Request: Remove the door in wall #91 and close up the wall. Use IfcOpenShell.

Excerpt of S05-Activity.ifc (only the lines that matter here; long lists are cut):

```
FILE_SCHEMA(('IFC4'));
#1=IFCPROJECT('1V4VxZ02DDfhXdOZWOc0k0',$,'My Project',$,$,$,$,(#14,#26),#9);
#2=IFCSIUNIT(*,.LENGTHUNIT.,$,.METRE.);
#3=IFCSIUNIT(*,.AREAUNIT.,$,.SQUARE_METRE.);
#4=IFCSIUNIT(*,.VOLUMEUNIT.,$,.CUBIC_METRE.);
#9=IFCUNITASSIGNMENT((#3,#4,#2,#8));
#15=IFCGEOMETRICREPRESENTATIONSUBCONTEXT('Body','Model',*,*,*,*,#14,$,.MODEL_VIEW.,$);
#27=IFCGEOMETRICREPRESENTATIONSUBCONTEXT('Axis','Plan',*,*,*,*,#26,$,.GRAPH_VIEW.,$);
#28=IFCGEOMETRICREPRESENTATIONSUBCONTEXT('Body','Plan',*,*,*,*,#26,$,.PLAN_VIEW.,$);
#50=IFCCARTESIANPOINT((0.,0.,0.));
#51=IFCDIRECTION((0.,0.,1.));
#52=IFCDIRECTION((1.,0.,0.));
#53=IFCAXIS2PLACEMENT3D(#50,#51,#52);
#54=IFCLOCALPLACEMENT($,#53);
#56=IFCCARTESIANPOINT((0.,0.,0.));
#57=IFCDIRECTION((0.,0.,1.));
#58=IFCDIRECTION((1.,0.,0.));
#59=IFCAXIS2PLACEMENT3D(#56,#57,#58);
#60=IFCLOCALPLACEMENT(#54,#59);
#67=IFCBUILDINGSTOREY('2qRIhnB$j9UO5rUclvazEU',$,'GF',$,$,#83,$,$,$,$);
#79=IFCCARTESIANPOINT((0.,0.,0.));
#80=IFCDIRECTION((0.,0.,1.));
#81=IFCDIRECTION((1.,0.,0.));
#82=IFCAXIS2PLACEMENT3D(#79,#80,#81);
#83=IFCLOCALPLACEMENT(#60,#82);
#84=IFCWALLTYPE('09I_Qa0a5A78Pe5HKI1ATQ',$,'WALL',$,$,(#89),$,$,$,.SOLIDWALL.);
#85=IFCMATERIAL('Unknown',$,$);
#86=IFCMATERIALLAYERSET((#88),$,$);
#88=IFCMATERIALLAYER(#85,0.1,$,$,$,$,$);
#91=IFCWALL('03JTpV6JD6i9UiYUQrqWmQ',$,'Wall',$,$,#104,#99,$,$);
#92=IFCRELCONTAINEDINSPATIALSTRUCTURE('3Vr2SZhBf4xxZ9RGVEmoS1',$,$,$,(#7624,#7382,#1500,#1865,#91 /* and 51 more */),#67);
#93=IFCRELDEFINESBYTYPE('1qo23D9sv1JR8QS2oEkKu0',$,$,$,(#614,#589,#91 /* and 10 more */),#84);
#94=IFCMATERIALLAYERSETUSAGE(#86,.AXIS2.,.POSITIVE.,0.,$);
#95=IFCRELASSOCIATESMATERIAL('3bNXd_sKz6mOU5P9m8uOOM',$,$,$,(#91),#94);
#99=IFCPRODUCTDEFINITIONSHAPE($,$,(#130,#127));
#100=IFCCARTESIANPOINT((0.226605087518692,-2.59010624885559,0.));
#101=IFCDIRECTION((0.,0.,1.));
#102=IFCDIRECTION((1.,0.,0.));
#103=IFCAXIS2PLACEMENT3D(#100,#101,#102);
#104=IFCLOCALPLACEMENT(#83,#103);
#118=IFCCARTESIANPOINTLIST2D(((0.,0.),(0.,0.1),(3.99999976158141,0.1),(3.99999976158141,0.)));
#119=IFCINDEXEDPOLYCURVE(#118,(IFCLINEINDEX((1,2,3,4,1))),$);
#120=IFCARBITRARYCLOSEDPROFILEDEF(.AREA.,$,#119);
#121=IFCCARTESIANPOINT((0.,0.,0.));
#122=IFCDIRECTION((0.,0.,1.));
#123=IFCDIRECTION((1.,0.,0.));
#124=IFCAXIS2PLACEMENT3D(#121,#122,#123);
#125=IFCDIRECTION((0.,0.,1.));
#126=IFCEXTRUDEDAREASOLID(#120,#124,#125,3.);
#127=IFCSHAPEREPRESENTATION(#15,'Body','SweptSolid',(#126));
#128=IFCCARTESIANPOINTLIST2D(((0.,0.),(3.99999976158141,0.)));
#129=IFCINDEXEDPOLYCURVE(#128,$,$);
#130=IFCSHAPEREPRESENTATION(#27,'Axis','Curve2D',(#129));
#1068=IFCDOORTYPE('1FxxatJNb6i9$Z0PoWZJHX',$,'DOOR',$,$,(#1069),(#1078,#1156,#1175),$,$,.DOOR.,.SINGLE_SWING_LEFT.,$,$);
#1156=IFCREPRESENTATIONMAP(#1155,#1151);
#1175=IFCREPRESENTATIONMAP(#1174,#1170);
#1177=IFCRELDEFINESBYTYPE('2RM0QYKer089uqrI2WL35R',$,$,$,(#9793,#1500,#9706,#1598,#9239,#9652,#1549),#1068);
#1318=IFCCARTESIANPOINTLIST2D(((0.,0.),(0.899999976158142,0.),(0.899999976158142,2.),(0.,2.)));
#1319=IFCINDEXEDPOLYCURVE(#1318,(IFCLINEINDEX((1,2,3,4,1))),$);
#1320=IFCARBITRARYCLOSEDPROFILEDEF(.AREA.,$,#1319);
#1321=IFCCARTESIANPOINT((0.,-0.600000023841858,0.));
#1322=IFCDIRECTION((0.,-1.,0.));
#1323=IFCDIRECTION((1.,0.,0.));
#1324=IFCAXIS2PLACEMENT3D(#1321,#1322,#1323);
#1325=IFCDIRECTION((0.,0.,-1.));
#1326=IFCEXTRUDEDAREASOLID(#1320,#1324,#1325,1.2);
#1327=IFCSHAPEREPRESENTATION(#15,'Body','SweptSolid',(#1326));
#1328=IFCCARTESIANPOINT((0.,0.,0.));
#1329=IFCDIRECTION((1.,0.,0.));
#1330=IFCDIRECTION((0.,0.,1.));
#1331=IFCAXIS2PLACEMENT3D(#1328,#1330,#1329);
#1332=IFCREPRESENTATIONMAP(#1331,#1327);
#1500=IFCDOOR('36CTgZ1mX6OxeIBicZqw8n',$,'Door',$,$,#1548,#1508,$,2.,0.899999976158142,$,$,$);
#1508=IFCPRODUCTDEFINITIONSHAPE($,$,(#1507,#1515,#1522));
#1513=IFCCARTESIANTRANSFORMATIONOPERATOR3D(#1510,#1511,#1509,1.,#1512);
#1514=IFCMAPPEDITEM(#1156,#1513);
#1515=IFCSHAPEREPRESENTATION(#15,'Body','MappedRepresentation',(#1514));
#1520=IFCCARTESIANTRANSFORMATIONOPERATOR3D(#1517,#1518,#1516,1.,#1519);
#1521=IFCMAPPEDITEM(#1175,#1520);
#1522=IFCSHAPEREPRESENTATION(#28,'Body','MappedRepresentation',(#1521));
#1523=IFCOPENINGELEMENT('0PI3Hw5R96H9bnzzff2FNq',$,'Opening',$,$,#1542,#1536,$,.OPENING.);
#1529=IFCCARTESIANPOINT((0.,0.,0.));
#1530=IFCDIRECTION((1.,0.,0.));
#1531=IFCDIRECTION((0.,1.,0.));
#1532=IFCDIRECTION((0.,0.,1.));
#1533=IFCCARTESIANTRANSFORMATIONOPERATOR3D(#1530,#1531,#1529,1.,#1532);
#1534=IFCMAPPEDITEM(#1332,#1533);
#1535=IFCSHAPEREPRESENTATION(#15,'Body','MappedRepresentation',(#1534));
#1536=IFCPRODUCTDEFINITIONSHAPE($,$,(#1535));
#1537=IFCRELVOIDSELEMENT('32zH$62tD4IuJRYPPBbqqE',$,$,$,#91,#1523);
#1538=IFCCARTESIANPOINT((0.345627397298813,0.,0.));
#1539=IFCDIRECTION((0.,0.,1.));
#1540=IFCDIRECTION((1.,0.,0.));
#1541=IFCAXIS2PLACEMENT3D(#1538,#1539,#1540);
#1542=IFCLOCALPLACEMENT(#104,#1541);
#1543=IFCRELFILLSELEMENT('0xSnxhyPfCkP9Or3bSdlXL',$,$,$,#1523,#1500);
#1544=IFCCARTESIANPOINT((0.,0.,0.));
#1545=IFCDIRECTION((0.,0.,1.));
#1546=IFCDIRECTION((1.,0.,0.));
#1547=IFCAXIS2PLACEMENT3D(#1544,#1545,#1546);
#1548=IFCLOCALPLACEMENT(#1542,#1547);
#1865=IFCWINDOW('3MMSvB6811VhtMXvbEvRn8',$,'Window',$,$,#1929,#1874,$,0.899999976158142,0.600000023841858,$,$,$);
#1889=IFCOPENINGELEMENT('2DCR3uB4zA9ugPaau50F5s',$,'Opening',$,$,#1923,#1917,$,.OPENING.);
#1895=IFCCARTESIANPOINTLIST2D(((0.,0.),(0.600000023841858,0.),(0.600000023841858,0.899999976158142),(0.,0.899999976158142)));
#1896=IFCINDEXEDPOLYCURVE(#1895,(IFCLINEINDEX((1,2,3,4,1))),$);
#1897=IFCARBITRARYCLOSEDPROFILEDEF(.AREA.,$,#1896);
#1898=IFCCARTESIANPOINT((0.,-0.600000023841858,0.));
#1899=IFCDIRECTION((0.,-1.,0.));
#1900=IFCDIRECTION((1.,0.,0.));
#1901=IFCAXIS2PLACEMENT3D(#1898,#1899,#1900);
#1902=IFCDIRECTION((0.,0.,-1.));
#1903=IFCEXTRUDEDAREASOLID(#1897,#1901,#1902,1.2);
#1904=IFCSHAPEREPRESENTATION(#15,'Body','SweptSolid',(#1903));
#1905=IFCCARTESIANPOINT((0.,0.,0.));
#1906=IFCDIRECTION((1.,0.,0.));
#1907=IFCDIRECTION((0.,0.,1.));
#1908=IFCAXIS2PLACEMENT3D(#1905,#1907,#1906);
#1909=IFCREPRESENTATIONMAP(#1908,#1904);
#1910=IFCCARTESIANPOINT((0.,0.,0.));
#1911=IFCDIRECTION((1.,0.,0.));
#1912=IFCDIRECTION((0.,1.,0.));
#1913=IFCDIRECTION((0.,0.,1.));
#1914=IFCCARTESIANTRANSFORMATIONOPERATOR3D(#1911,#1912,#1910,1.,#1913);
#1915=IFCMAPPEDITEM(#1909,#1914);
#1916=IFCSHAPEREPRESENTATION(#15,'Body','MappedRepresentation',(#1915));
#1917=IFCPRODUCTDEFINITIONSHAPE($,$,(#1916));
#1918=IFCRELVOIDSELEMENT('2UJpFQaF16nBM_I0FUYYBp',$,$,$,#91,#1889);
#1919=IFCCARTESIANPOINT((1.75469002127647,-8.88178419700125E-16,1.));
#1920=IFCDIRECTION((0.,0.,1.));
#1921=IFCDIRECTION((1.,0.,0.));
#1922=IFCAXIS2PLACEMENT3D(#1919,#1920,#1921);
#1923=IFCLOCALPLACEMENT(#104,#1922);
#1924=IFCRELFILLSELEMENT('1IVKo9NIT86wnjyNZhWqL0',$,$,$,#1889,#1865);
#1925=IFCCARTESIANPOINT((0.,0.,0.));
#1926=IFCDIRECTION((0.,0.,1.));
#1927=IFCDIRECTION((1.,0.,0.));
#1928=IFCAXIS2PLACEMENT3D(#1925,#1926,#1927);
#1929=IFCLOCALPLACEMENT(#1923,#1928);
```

```python
import ifcopenshell
import ifcopenshell.api.feature
import ifcopenshell.api.root
import ifcopenshell.geom
import ifcopenshell.util.shape

model = ifcopenshell.open("S05-Activity.ifc")
settings = ifcopenshell.geom.settings()


def volume(element):
    """Net volume in cubic metres, openings subtracted."""
    shape = ifcopenshell.geom.create_shape(settings, element)
    return ifcopenshell.util.shape.get_volume(shape.geometry)


door = model.by_guid("36CTgZ1mX6OxeIBicZqw8n")
opening = door.FillsVoids[0].RelatingOpeningElement
wall = opening.VoidsElements[0].RelatingBuildingElement
before = volume(wall)

ifcopenshell.api.root.remove_product(model, product=door)
ifcopenshell.api.feature.remove_feature(model, feature=opening)

after = volume(wall)

print(f"wall volume {before:.3f} -> {after:.3f} m3")

model.write("S05-Activity_v2.ifc")
```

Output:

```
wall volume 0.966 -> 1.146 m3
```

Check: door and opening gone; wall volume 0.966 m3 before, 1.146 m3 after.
